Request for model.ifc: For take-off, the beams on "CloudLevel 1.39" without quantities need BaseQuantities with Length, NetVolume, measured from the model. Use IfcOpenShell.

First a look at what the model holds.

```python
import ifcopenshell
import ifcopenshell.util.element
import ifcopenshell.util.unit

model = ifcopenshell.open("model.ifc")
print(model.schema)
for unit_type in ("LENGTHUNIT", "AREAUNIT", "VOLUMEUNIT"):
    print(unit_type, ifcopenshell.util.unit.calculate_unit_scale(model, unit_type))
storey = next(s for s in model.by_type("IfcBuildingStorey") if s.Name == "CloudLevel 1.39")
beams = [e for e in ifcopenshell.util.element.get_decomposition(storey) if e.is_a("IfcBeam")]
for e in sorted(beams, key=lambda e: e.id()):
    print(e.id(), e.is_a(), e.Name, list(ifcopenshell.util.element.get_psets(e, qtos_only=True)), sep=" | ")
```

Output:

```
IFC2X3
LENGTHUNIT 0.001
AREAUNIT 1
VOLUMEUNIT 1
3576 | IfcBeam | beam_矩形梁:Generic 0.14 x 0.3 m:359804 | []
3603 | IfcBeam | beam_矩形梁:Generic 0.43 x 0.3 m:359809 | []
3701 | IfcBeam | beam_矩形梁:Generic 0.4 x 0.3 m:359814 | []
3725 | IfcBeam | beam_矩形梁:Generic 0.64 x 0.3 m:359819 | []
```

```python
import ifcopenshell
import ifcopenshell.api.pset
import ifcopenshell.geom
import ifcopenshell.util.element
import ifcopenshell.util.shape
import ifcopenshell.util.unit

model = ifcopenshell.open("model.ifc")
unit_scale = ifcopenshell.util.unit.calculate_unit_scale(model)
volume_scale = ifcopenshell.util.unit.calculate_unit_scale(model, "VOLUMEUNIT")
settings = ifcopenshell.geom.settings()

storey = next(s for s in model.by_type("IfcBuildingStorey") if s.Name == "CloudLevel 1.39")
beams = [e for e in ifcopenshell.util.element.get_decomposition(storey) if e.is_a("IfcBeam")]

for e in sorted(beams, key=lambda e: e.id()):
    if ifcopenshell.util.element.get_psets(e, qtos_only=True, should_inherit=False):
        continue
    # Geometry comes back in metres, in the element's own axes.
    shape = ifcopenshell.geom.create_shape(settings, e)
    values = {
        "Length": ifcopenshell.util.shape.get_max_xyz(shape.geometry) / unit_scale,
        "NetVolume": ifcopenshell.util.shape.get_volume(shape.geometry) / volume_scale,
    }
    qto = ifcopenshell.api.pset.add_qto(model, product=e, name="BaseQuantities")
    ifcopenshell.api.pset.edit_qto(model, qto=qto, properties=values)
    print(e.id(), {k: round(v, 3) for k, v in values.items()})

model.write("model_updated.ifc")
```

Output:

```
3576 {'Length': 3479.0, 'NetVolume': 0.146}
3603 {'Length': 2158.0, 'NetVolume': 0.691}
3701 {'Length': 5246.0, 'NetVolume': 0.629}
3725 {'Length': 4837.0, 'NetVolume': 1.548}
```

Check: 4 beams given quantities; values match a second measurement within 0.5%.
